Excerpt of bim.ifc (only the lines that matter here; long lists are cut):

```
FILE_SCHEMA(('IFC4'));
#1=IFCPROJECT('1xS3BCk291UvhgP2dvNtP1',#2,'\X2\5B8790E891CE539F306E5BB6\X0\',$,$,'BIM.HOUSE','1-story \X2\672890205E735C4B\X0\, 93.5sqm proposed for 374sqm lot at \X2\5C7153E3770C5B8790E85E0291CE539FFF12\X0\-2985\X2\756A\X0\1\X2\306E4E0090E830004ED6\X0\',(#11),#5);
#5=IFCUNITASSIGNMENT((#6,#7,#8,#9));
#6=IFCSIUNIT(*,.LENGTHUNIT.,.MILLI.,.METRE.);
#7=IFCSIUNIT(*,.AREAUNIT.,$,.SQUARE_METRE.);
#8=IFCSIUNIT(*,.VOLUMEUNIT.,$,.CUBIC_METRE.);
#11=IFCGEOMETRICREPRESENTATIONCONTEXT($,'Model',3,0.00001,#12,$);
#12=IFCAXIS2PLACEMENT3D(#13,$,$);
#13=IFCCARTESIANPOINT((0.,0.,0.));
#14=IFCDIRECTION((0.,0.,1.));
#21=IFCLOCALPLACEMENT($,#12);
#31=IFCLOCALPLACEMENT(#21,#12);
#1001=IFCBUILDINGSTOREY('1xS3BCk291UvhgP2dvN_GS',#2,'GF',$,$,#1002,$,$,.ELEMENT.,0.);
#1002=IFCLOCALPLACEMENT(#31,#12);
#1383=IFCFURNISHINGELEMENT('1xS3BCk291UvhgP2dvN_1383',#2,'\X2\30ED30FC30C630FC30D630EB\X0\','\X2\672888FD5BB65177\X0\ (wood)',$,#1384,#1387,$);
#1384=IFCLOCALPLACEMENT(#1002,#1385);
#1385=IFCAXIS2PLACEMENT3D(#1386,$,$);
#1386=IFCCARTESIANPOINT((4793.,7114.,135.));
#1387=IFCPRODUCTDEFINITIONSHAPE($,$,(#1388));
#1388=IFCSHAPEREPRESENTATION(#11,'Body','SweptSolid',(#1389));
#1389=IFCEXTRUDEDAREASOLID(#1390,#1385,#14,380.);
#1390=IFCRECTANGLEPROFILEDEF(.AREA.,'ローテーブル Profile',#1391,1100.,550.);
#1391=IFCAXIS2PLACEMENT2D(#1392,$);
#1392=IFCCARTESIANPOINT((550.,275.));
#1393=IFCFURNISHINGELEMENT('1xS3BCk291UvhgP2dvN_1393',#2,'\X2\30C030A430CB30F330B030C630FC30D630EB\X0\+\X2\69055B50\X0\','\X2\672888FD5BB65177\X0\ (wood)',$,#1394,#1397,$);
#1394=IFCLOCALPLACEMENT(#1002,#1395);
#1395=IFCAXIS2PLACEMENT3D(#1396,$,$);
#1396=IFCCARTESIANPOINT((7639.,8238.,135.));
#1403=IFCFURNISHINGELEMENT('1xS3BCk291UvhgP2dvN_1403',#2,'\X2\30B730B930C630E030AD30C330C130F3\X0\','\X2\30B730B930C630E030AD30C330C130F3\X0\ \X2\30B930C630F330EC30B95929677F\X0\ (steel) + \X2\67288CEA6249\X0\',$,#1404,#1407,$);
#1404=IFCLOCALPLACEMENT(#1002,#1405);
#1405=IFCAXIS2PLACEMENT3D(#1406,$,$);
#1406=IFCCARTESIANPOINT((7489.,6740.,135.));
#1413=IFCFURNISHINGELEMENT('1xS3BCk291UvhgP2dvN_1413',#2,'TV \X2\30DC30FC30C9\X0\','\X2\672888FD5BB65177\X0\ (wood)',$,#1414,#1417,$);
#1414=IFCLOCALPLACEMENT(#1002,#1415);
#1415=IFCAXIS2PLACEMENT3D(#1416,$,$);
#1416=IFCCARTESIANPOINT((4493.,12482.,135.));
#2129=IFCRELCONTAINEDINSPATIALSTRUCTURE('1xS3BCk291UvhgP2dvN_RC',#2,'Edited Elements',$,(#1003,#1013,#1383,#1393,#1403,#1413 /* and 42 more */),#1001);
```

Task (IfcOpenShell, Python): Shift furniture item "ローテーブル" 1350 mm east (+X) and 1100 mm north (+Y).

```python
import ifcopenshell
import ifcopenshell.api.geometry
import ifcopenshell.util.placement
import ifcopenshell.util.unit

model = ifcopenshell.open("bim.ifc")
unit_scale = ifcopenshell.util.unit.calculate_unit_scale(model)

item = model.by_guid("1xS3BCk291UvhgP2dvN_1383")
matrix = ifcopenshell.util.placement.get_local_placement(item.ObjectPlacement)
matrix[0, 3] += 1.35 / unit_scale
matrix[1, 3] += 1.1 / unit_scale
ifcopenshell.api.geometry.edit_object_placement(model, product=item, matrix=matrix, is_si=False)

print(ifcopenshell.util.placement.get_local_placement(item.ObjectPlacement).round(3) + 0.0)

model.write("bim-out.ifc")
```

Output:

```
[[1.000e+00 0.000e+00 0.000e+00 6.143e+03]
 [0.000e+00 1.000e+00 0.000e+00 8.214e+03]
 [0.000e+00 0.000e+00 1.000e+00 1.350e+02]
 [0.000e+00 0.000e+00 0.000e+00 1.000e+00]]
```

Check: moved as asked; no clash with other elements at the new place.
